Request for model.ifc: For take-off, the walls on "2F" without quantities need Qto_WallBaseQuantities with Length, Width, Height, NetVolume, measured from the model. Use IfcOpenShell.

First a look at what the model holds.

```python
import ifcopenshell
import ifcopenshell.util.element
import ifcopenshell.util.unit

model = ifcopenshell.open("model.ifc")
print(model.schema)
for unit_type in ("LENGTHUNIT", "AREAUNIT", "VOLUMEUNIT"):
    print(unit_type, ifcopenshell.util.unit.calculate_unit_scale(model, unit_type))
storey = next(s for s in model.by_type("IfcBuildingStorey") if s.Name == "2F")
walls = [e for e in ifcopenshell.util.element.get_decomposition(storey) if e.is_a("IfcWall")]
for e in sorted(walls, key=lambda e: e.id()):
    print(e.id(), e.is_a(), e.Name, list(ifcopenshell.util.element.get_psets(e, qtos_only=True)), sep=" | ")
```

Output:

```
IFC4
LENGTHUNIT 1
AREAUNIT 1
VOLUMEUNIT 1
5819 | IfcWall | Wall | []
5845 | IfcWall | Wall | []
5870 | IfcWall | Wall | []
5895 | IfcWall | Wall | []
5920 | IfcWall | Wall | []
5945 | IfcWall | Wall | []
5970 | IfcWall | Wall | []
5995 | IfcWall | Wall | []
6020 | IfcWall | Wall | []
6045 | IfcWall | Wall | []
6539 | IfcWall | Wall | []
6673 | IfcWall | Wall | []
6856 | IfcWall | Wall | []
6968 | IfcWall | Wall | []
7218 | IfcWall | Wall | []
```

```python
import ifcopenshell
import ifcopenshell.api.pset
import ifcopenshell.geom
import ifcopenshell.util.element
import ifcopenshell.util.shape
import ifcopenshell.util.unit

model = ifcopenshell.open("model.ifc")
unit_scale = ifcopenshell.util.unit.calculate_unit_scale(model)
volume_scale = ifcopenshell.util.unit.calculate_unit_scale(model, "VOLUMEUNIT")
settings = ifcopenshell.geom.settings()

storey = next(s for s in model.by_type("IfcBuildingStorey") if s.Name == "2F")
walls = [e for e in ifcopenshell.util.element.get_decomposition(storey) if e.is_a("IfcWall")]

for e in sorted(walls, key=lambda e: e.id()):
    if ifcopenshell.util.element.get_psets(e, qtos_only=True, should_inherit=False):
        continue
    # Geometry comes back in metres, in the element's own axes.
    shape = ifcopenshell.geom.create_shape(settings, e)
    values = {
        "Length": ifcopenshell.util.shape.get_x(shape.geometry) / unit_scale,
        "Width": ifcopenshell.util.shape.get_y(shape.geometry) / unit_scale,
        "Height": ifcopenshell.util.shape.get_z(shape.geometry) / unit_scale,
        "NetVolume": ifcopenshell.util.shape.get_volume(shape.geometry) / volume_scale,
    }
    qto = ifcopenshell.api.pset.add_qto(model, product=e, name="Qto_WallBaseQuantities")
    ifcopenshell.api.pset.edit_qto(model, qto=qto, properties=values)
    print(e.id(), {k: round(v, 3) for k, v in values.items()})

model.write("model_edited.ifc")
```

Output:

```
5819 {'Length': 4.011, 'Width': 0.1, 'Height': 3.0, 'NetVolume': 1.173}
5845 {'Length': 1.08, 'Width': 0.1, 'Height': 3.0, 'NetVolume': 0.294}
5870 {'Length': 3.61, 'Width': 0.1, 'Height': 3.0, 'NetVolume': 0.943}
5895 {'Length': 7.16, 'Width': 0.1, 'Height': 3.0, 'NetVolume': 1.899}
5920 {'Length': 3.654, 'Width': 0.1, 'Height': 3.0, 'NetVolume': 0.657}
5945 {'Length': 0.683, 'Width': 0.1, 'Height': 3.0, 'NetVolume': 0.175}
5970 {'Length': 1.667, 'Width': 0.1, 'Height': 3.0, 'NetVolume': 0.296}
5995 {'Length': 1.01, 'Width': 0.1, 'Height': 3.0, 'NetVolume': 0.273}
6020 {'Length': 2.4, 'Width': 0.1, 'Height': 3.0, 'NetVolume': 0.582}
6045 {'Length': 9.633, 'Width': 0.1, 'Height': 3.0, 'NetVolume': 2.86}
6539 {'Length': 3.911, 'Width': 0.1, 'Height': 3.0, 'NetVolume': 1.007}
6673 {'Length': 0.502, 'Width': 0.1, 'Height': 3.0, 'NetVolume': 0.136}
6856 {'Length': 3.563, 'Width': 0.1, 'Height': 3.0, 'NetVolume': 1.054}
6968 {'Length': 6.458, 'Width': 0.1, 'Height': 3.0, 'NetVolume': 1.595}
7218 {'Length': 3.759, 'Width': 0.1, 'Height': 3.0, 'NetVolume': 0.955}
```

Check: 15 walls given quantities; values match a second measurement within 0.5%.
